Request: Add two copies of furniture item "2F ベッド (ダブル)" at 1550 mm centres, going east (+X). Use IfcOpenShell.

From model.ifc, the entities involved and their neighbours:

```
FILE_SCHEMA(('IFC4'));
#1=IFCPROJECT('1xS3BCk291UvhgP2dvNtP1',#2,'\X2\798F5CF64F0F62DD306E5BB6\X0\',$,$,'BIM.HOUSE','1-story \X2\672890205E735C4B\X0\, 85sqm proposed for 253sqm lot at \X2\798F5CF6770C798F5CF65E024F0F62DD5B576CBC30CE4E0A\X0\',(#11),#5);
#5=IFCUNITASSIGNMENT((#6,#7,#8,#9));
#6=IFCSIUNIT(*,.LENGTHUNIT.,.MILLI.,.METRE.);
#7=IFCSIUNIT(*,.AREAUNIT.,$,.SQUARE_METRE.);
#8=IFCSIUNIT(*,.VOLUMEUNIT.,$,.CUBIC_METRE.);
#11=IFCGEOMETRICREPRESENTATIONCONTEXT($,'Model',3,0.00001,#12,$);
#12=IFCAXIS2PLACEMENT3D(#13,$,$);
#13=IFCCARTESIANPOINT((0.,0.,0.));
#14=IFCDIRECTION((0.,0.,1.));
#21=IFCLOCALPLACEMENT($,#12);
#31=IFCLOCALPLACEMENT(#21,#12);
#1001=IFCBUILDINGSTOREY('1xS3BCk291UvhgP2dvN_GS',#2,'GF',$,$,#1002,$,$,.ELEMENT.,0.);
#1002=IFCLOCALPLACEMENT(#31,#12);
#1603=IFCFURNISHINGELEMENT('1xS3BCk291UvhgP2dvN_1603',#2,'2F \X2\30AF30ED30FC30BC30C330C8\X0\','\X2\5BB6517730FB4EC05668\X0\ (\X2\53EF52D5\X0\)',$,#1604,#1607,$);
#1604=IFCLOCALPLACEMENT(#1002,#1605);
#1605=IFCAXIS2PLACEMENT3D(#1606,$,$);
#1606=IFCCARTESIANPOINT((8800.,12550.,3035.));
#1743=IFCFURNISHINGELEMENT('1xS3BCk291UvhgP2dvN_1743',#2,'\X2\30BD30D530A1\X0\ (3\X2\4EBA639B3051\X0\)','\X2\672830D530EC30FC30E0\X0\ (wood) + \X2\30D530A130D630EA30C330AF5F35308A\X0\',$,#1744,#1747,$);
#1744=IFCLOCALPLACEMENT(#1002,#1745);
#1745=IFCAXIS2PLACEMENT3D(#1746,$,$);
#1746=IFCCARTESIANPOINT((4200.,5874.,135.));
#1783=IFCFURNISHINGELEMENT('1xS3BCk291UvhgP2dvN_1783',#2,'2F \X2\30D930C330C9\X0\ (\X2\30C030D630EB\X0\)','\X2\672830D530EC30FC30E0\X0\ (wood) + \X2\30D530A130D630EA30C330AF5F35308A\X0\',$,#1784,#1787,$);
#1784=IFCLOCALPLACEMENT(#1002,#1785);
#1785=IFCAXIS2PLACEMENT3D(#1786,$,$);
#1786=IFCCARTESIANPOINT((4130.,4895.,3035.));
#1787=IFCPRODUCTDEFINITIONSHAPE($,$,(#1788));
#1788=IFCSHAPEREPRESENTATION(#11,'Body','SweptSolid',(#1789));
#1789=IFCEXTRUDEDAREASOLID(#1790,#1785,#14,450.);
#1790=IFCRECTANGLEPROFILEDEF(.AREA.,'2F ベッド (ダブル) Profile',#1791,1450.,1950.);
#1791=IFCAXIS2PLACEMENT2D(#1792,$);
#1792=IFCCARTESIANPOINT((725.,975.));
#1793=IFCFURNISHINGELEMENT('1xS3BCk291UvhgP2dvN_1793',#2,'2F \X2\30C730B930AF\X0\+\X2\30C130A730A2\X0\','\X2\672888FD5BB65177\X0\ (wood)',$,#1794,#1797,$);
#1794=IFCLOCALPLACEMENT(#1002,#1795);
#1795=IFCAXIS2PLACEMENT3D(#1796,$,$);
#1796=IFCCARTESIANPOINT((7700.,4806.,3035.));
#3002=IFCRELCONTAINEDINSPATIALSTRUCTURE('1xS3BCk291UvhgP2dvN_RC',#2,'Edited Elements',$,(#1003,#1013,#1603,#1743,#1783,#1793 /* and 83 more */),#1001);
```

```python
import numpy as np
import ifcopenshell
import ifcopenshell.api.geometry
import ifcopenshell.api.root
import ifcopenshell.util.element
import ifcopenshell.util.placement
import ifcopenshell.util.unit

model = ifcopenshell.open("model.ifc")
unit_scale = ifcopenshell.util.unit.calculate_unit_scale(model)


def reuse_history(source, copy):
    """copy_class also copies each property set's owner history, people and application; keep the originals."""
    for rel in copy.IsDefinedBy:
        if rel.is_a("IfcRelDefinesByProperties") and (history := rel.RelatingPropertyDefinition.OwnerHistory):
            rel.RelatingPropertyDefinition.OwnerHistory = source.OwnerHistory
            ifcopenshell.util.element.remove_deep2(model, history)


source = model.by_guid("1xS3BCk291UvhgP2dvN_1783")
base = ifcopenshell.util.placement.get_local_placement(source.ObjectPlacement)
step = np.array([1.0, 0.0, 0.0]) * 1.55 / unit_scale

for i in range(1, 3):
    copy = ifcopenshell.api.root.copy_class(model, product=source)
    copy.Representation = ifcopenshell.util.element.copy_deep(
        model, source.Representation, exclude=["IfcGeometricRepresentationContext", "IfcRepresentationMap"]
    )
    reuse_history(source, copy)
    matrix = base.copy()
    matrix[:3, 3] += i * step
    print("added at", matrix[:3, 3].round(3) + 0.0)
    ifcopenshell.api.geometry.edit_object_placement(model, product=copy, matrix=matrix, is_si=False)

model.write("model_updated.ifc")
```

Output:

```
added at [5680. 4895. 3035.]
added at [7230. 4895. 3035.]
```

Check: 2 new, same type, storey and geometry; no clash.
